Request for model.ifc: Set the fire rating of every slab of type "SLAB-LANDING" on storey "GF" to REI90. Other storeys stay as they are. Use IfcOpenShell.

First a look at what the model holds.

```python
import ifcopenshell
import ifcopenshell.util.element

model = ifcopenshell.open("model.ifc")
print(model.schema)
storey = next(s for s in model.by_type("IfcBuildingStorey") if s.Name == "GF")
slabs = [e for e in ifcopenshell.util.element.get_decomposition(storey) if e.is_a("IfcSlab")]
seen = {}
for e in slabs:
    element_type = ifcopenshell.util.element.get_type(e)
    key = (element_type.Name if element_type != e and element_type else None, ifcopenshell.util.element.get_pset(e, "Pset_SlabCommon", "FireRating"))
    seen[key] = seen.get(key, 0) + 1
for (name, value), count in sorted(seen.items(), key=str):
    print(count, "x", name, "|", value)
```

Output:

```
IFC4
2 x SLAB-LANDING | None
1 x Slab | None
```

```python
import ifcopenshell
import ifcopenshell.api.pset
import ifcopenshell.util.element

model = ifcopenshell.open("model.ifc")

storey = next(s for s in model.by_type("IfcBuildingStorey") if s.Name == "GF")
slabs = [e for e in ifcopenshell.util.element.get_decomposition(storey) if e.is_a("IfcSlab")]

count = 0
for e in slabs:
    element_type = ifcopenshell.util.element.get_type(e)
    if element_type in (None, e) or element_type.Name != "SLAB-LANDING":
        continue
    # add_pset returns the element's existing set when there is one.
    pset = ifcopenshell.api.pset.add_pset(model, product=e, name="Pset_SlabCommon")
    ifcopenshell.api.pset.edit_pset(model, pset=pset, properties={"FireRating": "REI90"})
    count += 1

print(count, "slabs updated")

model.write("model_v2.ifc")
```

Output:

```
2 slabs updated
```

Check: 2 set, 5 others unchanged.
